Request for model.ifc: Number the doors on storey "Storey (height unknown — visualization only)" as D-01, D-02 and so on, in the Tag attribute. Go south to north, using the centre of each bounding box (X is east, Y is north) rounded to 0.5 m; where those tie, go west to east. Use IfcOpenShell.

First a look at what the model holds.

```python
import ifcopenshell
import ifcopenshell.util.element
import ifcopenshell.util.placement

model = ifcopenshell.open("model.ifc")
print(model.schema)
storey = next(s for s in model.by_type("IfcBuildingStorey") if s.Name == "Storey (height unknown — visualization only)")
doors = [e for e in ifcopenshell.util.element.get_decomposition(storey) if e.is_a("IfcDoor")]
for e in sorted(doors, key=lambda e: e.id()):
    origin = ifcopenshell.util.placement.get_local_placement(e.ObjectPlacement)[:3, 3]
    print(e.id(), e.Tag, e.Name, origin.round(2) + 0.0, sep=" | ")
```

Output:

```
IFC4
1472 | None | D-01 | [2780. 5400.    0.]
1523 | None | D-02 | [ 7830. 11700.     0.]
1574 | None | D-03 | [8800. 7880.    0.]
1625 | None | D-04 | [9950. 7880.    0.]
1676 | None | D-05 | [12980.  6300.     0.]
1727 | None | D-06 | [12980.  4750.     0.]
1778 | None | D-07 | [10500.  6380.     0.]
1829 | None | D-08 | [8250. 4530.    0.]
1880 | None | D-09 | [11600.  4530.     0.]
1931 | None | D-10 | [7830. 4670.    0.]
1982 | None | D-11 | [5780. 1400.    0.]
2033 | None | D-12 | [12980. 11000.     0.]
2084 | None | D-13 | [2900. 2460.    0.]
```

```python
import ifcopenshell
import ifcopenshell.geom
import ifcopenshell.util.element
import ifcopenshell.util.shape

model = ifcopenshell.open("model.ifc")
settings = ifcopenshell.geom.settings()
settings.set("use-world-coords", True)


def centre(element):
    shape = ifcopenshell.geom.create_shape(settings, element)
    return ifcopenshell.util.shape.get_bbox_centroid(shape.geometry)


storey = next(s for s in model.by_type("IfcBuildingStorey") if s.Name == "Storey (height unknown — visualization only)")
doors = [e for e in ifcopenshell.util.element.get_decomposition(storey) if e.is_a("IfcDoor")]

# Insertion points can sit at a corner or the storey origin, so sort by the geometry (in metres).
centres = {e: centre(e) for e in doors}
doors.sort(key=lambda e: (round(centres[e][1] / 0.5), centres[e][0]))

for i, e in enumerate(doors, start=1):
    number = f"D-{i:02d}"
    e.Tag = number
    print(e.id(), number)

model.write("model_edited.ifc")
```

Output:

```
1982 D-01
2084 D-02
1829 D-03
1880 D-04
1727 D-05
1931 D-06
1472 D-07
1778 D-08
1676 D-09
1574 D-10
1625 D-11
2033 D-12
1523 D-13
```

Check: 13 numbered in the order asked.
